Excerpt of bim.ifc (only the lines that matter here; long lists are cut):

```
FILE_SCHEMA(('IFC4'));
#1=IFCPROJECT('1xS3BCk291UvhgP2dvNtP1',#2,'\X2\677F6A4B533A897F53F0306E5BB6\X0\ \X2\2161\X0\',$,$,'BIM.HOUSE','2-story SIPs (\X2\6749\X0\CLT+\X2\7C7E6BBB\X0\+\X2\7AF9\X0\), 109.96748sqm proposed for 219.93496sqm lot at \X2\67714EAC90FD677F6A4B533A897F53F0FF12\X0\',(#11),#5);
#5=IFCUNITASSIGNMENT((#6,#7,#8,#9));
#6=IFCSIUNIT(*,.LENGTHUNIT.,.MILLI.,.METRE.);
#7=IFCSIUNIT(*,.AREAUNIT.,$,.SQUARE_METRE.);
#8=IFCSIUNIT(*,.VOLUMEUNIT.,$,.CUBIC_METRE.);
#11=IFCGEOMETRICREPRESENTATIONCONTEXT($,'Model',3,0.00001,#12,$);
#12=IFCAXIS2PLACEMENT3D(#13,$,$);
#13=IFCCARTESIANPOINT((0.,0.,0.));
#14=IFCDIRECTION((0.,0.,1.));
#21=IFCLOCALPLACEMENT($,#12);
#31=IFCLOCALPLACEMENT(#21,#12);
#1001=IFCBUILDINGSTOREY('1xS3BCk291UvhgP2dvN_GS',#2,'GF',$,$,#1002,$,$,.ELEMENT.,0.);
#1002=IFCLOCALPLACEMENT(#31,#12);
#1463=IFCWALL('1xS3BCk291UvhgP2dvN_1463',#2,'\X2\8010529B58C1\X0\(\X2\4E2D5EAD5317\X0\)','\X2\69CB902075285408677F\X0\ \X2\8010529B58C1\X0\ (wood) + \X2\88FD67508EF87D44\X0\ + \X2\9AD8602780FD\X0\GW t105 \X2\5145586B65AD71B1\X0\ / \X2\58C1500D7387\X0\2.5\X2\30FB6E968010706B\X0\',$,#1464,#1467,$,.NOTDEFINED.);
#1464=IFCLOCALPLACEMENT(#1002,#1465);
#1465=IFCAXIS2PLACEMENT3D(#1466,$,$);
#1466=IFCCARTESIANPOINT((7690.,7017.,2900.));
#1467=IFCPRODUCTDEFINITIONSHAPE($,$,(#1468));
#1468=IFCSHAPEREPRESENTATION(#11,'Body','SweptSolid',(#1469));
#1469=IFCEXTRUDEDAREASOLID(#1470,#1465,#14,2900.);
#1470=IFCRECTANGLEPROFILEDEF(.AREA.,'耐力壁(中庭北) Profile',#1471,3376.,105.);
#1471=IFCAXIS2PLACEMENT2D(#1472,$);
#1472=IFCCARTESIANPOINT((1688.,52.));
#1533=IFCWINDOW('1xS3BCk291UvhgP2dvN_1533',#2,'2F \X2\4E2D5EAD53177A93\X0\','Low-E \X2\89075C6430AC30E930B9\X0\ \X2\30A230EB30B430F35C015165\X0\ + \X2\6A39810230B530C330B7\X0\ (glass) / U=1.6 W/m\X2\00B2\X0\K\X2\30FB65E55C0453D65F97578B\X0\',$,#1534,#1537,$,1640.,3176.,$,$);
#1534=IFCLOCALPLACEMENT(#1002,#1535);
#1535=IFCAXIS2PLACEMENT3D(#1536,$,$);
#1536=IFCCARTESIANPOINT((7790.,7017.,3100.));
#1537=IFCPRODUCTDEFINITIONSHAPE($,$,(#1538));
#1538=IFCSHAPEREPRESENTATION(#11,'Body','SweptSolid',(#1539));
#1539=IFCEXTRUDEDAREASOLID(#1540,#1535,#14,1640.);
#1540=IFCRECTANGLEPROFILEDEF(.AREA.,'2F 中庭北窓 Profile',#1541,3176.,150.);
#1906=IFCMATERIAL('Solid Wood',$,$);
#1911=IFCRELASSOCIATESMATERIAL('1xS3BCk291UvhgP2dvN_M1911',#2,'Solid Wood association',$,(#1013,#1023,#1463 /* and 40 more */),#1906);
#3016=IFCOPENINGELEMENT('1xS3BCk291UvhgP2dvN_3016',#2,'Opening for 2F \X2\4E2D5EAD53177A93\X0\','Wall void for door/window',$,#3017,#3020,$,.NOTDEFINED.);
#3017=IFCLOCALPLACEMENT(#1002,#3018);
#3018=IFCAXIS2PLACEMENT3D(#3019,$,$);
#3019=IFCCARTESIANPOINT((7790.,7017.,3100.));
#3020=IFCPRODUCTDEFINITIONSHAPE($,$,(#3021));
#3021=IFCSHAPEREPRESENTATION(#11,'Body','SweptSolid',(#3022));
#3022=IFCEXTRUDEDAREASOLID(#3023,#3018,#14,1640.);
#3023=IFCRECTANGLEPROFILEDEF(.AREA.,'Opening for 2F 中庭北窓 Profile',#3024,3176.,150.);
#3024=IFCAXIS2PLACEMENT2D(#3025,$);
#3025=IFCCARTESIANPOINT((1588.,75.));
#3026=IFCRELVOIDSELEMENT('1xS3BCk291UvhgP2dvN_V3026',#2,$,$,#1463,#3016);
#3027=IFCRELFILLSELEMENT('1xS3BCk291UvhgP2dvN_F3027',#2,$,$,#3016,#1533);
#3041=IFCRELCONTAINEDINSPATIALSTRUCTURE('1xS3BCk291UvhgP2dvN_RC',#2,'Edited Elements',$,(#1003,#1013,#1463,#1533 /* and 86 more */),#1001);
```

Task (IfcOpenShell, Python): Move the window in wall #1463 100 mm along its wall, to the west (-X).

```python
import ifcopenshell
import ifcopenshell.api.geometry
import ifcopenshell.util.placement
import ifcopenshell.util.unit

model = ifcopenshell.open("bim.ifc")
unit_scale = ifcopenshell.util.unit.calculate_unit_scale(model)

window = model.by_guid("1xS3BCk291UvhgP2dvN_1533")
opening = window.FillsVoids[0].RelatingOpeningElement
wall = opening.VoidsElements[0].RelatingBuildingElement

wall_matrix = ifcopenshell.util.placement.get_local_placement(wall.ObjectPlacement)
shift = wall_matrix[:3, 0] * -0.1 / unit_scale
before = ifcopenshell.util.placement.get_local_placement(window.ObjectPlacement)[:3, 3].copy()

# The window is not placed relative to its opening, so move both.
for product in (opening, window):
    matrix = ifcopenshell.util.placement.get_local_placement(product.ObjectPlacement)
    matrix[:3, 3] += shift
    ifcopenshell.api.geometry.edit_object_placement(model, product=product, matrix=matrix, is_si=False)

after = ifcopenshell.util.placement.get_local_placement(window.ObjectPlacement)[:3, 3]
print("window moved by", (after - before).round(3) + 0.0)

model.write("bim_rev.ifc")
```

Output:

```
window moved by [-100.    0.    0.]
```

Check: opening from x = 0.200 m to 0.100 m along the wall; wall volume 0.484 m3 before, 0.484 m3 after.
